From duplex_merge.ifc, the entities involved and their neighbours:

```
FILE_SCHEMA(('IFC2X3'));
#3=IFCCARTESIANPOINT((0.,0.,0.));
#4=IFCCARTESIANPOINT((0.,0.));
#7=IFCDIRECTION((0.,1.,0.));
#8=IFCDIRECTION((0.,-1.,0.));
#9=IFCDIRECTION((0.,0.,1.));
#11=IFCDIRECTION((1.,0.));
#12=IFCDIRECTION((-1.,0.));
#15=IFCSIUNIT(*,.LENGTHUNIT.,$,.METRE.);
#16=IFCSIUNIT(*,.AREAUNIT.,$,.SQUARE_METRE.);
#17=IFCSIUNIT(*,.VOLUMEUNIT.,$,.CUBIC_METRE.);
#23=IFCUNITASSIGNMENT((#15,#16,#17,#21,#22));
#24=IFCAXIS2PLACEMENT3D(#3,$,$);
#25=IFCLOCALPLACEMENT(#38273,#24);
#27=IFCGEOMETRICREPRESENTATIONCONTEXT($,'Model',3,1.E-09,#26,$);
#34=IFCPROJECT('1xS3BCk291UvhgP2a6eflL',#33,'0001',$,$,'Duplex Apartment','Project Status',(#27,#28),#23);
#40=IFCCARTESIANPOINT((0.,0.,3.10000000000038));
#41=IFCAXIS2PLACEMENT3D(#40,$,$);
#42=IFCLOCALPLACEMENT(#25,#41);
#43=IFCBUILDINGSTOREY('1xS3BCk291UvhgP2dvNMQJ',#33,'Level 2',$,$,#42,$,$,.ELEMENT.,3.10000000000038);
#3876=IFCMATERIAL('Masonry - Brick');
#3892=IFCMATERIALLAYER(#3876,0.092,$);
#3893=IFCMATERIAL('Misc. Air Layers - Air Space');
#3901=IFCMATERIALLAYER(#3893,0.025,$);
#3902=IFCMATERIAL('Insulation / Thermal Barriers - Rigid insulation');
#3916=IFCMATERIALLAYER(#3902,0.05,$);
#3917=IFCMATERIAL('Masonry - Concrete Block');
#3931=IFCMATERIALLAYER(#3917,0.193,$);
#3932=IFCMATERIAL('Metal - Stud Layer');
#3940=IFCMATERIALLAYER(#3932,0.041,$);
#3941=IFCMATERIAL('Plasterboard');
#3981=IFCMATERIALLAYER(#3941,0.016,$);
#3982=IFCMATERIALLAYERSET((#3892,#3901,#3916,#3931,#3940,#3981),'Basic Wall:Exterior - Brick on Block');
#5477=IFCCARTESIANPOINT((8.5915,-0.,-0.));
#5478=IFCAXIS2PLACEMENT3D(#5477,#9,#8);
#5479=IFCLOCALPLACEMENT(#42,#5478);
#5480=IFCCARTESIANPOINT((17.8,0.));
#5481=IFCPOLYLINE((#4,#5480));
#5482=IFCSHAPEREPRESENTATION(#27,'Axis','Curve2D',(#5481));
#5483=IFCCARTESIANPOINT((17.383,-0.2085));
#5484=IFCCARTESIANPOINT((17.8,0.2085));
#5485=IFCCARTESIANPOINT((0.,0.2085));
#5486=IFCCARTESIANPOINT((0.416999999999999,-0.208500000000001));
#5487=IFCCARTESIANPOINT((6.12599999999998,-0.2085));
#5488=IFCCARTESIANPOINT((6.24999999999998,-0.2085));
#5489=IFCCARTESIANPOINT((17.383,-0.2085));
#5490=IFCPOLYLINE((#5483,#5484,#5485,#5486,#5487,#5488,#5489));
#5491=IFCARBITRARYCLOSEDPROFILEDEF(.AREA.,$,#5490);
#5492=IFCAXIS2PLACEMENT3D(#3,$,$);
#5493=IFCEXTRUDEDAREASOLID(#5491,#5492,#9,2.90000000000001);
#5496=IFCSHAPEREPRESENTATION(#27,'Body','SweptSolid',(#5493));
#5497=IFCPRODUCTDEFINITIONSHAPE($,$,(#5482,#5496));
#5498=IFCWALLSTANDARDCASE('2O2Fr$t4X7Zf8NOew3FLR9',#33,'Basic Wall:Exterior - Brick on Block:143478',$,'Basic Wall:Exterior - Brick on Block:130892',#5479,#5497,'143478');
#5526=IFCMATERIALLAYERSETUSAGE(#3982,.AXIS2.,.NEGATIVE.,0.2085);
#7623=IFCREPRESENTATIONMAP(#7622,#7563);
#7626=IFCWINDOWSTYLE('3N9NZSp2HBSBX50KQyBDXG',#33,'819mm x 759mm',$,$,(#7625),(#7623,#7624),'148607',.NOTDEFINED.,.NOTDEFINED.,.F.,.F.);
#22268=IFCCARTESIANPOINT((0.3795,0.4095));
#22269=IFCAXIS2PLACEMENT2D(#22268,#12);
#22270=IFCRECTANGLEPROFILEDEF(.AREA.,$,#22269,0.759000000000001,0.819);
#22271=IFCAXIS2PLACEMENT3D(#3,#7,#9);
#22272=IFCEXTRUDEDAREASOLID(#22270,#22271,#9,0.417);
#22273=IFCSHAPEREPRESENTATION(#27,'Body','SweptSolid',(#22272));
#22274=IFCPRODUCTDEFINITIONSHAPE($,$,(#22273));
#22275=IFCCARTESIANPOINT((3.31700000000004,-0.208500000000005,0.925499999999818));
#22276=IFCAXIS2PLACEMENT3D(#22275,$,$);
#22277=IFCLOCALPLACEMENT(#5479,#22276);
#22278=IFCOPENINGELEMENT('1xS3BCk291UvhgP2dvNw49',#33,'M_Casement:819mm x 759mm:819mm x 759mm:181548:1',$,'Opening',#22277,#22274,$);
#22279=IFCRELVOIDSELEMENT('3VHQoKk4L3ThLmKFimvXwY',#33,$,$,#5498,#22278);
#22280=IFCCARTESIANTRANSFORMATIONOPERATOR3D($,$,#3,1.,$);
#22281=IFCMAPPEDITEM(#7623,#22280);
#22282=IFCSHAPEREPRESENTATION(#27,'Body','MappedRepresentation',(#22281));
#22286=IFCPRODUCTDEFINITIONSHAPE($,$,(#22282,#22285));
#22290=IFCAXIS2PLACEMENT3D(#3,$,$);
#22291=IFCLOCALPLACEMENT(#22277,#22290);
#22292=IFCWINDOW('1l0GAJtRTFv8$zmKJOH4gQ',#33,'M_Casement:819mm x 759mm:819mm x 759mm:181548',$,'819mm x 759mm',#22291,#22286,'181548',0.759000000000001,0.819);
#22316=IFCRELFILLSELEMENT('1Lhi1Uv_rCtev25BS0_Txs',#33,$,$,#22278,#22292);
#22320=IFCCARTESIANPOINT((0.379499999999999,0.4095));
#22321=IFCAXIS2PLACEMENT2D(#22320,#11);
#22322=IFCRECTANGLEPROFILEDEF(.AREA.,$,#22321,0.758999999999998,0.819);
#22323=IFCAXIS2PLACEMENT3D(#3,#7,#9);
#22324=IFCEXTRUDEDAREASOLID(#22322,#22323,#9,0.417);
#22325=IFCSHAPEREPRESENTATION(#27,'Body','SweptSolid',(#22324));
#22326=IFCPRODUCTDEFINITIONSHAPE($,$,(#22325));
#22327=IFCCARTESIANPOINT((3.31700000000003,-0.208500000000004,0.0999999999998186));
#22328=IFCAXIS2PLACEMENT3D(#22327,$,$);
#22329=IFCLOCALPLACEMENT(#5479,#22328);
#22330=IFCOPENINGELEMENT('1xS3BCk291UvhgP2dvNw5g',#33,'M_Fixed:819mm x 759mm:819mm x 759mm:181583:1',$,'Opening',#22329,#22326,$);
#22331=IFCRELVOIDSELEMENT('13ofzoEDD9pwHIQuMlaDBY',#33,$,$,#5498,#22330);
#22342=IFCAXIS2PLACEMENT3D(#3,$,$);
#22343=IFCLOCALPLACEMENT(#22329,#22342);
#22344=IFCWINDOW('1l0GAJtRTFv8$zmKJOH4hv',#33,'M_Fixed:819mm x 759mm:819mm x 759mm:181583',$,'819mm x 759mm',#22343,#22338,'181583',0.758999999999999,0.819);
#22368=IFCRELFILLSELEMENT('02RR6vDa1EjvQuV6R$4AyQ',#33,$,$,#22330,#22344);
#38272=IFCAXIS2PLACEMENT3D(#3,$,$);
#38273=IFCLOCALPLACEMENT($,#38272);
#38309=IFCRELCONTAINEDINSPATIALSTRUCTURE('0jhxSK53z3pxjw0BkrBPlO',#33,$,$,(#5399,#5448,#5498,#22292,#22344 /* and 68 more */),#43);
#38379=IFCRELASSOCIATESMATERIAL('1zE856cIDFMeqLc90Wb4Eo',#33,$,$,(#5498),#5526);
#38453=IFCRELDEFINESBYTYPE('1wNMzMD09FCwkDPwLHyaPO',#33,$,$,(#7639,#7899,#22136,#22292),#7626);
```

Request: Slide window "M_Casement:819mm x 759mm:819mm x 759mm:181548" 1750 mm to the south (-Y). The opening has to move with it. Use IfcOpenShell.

```python
import ifcopenshell
import ifcopenshell.api.geometry
import ifcopenshell.util.placement

model = ifcopenshell.open("duplex_merge.ifc")

window = model.by_guid("1l0GAJtRTFv8$zmKJOH4gQ")
opening = window.FillsVoids[0].RelatingOpeningElement
wall = opening.VoidsElements[0].RelatingBuildingElement

wall_matrix = ifcopenshell.util.placement.get_local_placement(wall.ObjectPlacement)
shift = wall_matrix[:3, 0] * 1.75
before = ifcopenshell.util.placement.get_local_placement(window.ObjectPlacement)[:3, 3].copy()

# The window is placed relative to its opening, so it follows when the opening moves.
matrix = ifcopenshell.util.placement.get_local_placement(opening.ObjectPlacement)
matrix[:3, 3] += shift
ifcopenshell.api.geometry.edit_object_placement(
    model, product=opening, matrix=matrix, is_si=False, should_transform_children=True
)

after = ifcopenshell.util.placement.get_local_placement(window.ObjectPlacement)[:3, 3]
print("window moved by", (after - before).round(3) + 0.0)

model.write("duplex_merge-out.ifc")
```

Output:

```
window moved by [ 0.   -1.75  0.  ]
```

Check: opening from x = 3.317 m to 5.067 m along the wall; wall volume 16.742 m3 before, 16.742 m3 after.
